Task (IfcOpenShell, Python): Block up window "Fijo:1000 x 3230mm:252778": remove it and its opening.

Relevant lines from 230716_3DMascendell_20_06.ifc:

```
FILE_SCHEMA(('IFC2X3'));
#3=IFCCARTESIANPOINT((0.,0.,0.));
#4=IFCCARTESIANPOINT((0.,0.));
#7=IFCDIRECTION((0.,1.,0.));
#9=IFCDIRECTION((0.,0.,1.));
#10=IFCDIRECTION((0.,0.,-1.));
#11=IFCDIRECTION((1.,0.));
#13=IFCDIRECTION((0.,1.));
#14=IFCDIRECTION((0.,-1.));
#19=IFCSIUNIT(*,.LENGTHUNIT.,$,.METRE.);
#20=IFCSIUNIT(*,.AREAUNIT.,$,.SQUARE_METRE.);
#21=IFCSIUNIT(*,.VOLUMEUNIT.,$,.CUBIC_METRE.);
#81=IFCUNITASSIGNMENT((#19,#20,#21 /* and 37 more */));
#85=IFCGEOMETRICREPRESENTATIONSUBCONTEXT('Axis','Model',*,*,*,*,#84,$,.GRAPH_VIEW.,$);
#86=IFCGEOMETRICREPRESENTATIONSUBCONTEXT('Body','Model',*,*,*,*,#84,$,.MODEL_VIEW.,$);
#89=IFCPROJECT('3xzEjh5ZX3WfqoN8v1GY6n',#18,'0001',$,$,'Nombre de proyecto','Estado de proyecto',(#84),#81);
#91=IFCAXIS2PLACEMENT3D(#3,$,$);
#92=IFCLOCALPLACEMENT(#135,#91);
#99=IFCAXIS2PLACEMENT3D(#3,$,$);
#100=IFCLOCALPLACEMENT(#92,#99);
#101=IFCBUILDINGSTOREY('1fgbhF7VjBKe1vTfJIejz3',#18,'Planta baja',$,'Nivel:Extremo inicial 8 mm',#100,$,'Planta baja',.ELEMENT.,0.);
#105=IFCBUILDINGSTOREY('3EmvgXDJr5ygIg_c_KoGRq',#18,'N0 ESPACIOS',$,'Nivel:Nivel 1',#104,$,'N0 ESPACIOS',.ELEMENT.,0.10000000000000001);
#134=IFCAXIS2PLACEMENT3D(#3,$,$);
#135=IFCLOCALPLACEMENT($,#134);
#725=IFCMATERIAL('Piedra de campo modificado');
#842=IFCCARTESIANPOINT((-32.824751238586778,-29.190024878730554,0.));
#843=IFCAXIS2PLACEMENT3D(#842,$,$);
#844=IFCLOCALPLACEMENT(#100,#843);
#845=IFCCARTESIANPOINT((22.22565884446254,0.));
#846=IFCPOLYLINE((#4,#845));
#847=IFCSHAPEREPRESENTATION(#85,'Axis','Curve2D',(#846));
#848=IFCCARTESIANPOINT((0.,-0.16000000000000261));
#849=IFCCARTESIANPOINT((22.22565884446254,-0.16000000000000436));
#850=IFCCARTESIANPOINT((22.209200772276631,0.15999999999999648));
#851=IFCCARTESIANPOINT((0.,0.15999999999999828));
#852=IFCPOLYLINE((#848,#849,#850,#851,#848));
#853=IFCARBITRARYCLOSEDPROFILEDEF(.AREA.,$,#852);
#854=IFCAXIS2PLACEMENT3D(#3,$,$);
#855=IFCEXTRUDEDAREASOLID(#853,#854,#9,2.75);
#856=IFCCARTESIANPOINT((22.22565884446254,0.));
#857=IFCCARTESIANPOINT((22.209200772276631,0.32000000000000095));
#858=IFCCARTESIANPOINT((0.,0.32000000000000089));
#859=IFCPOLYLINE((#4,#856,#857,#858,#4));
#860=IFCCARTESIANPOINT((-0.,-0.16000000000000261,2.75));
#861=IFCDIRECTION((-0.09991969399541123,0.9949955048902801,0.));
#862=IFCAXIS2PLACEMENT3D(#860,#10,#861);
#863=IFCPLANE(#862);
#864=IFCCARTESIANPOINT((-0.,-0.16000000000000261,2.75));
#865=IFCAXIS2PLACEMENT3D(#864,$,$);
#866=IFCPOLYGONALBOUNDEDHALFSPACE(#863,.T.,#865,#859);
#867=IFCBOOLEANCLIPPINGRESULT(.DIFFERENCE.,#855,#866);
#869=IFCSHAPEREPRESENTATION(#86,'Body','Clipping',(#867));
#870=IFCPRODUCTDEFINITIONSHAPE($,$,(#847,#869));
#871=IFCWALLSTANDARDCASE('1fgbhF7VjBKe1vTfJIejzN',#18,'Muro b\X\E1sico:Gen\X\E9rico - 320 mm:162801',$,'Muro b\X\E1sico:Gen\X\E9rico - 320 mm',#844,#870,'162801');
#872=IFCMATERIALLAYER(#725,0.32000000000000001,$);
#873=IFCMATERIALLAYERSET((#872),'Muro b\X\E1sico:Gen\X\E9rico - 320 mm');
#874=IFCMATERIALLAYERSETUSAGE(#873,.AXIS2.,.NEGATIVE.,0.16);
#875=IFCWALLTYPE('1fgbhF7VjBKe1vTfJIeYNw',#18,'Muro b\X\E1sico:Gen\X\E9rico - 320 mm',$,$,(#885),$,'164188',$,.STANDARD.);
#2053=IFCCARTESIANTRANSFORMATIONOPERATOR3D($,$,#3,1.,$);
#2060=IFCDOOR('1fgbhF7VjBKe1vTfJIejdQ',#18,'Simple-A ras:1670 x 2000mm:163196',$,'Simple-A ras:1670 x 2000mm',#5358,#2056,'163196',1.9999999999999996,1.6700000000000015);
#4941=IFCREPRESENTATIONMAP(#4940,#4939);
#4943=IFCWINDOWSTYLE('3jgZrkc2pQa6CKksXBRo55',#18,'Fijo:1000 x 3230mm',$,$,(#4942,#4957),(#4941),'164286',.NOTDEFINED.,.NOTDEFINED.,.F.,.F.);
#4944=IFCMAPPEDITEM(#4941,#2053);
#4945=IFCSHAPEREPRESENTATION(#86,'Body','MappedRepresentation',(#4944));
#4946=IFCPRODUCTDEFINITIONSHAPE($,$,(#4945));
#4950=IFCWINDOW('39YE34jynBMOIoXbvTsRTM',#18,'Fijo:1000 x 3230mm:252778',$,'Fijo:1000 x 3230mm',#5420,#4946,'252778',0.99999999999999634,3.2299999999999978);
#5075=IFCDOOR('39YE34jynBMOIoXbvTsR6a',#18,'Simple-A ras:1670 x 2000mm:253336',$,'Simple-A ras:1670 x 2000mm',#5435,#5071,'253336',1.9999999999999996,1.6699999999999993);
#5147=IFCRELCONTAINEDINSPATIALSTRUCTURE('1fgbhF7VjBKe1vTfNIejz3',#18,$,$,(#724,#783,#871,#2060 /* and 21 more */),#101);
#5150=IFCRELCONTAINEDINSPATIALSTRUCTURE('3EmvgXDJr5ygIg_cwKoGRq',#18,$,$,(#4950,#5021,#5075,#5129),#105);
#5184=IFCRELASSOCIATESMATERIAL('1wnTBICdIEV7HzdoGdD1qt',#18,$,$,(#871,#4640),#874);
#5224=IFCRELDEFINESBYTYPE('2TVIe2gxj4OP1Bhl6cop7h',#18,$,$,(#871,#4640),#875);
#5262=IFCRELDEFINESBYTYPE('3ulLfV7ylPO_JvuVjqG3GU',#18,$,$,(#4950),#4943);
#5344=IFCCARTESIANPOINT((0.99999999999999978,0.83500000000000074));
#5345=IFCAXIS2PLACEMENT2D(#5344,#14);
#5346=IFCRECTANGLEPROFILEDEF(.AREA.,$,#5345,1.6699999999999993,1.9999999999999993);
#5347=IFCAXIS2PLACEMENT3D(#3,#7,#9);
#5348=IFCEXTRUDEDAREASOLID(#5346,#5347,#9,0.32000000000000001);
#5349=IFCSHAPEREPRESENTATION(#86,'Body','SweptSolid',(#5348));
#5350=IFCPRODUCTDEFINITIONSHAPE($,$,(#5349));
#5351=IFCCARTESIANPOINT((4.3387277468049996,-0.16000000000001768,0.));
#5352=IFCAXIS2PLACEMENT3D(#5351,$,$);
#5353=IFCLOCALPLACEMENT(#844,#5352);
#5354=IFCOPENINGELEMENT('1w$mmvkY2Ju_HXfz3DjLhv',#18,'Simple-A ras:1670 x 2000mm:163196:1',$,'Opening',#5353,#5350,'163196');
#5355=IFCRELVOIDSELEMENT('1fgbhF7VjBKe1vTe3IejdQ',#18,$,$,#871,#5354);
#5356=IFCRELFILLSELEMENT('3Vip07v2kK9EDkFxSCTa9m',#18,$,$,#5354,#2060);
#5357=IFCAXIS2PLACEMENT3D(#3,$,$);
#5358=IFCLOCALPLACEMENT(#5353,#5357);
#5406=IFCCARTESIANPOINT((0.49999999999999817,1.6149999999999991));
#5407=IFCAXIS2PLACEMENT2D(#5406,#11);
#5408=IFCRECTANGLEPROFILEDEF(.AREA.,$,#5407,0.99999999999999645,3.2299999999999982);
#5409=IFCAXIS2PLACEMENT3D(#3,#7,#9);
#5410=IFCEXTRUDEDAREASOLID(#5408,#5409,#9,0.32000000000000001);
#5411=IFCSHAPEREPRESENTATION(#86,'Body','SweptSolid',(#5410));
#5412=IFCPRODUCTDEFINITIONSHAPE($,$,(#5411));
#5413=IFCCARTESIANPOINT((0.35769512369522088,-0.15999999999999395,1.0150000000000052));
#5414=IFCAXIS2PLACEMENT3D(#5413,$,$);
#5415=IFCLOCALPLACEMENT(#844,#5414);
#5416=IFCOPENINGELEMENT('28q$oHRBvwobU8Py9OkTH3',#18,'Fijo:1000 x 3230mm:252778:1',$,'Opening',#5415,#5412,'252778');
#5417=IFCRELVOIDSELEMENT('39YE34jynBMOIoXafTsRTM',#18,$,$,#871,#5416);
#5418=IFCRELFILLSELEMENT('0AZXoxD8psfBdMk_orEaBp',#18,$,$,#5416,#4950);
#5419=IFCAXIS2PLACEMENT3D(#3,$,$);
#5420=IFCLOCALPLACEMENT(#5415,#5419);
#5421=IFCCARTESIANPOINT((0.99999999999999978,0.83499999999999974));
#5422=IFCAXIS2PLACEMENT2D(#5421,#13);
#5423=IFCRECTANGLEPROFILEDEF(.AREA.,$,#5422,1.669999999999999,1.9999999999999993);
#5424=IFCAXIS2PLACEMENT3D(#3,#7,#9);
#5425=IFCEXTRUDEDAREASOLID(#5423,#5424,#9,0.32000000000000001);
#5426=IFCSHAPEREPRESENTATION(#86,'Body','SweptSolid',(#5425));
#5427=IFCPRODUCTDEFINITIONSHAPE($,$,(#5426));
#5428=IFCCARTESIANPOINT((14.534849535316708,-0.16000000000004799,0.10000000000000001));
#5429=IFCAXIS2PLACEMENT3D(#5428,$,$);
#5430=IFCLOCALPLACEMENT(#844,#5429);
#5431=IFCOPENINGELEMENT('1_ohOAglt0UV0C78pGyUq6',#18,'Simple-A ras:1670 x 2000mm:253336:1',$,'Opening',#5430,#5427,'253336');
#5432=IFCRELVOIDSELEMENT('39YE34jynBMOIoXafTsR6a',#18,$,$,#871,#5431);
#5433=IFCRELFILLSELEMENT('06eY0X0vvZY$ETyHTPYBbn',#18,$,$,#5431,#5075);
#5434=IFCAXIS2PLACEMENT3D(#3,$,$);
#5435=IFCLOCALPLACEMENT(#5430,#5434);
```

```python
import ifcopenshell
import ifcopenshell.api.feature
import ifcopenshell.api.root
import ifcopenshell.geom
import ifcopenshell.util.shape

model = ifcopenshell.open("230716_3DMascendell_20_06.ifc")
settings = ifcopenshell.geom.settings()


def volume(element):
    """Net volume in cubic metres, openings subtracted."""
    shape = ifcopenshell.geom.create_shape(settings, element)
    return ifcopenshell.util.shape.get_volume(shape.geometry)


window = model.by_guid("39YE34jynBMOIoXbvTsRTM")
opening = window.FillsVoids[0].RelatingOpeningElement
wall = opening.VoidsElements[0].RelatingBuildingElement
before = volume(wall)

ifcopenshell.api.root.remove_product(model, product=window)
ifcopenshell.api.feature.remove_feature(model, feature=opening)

after = volume(wall)

print(f"wall volume {before:.3f} -> {after:.3f} m3")

model.write("230716_3DMascendell_20_06_rev.ifc")
```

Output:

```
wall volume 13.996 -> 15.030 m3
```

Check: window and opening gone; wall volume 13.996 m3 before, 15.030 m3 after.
